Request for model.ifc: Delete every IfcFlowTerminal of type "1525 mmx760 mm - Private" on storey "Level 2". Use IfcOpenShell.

First a look at what the model holds.

```python
import ifcopenshell
import ifcopenshell.util.element

model = ifcopenshell.open("model.ifc")
print(model.schema)
storey = next(s for s in model.by_type("IfcBuildingStorey") if s.Name == "Level 2")
terminals = [e for e in ifcopenshell.util.element.get_decomposition(storey) if e.is_a("IfcFlowTerminal")]
seen = {}
for e in terminals:
    element_type = ifcopenshell.util.element.get_type(e)
    name = element_type.Name if element_type not in (None, e) else None
    seen[name] = seen.get(name, 0) + 1
for name, count in sorted(seen.items(), key=str):
    print(count, "x", name)
```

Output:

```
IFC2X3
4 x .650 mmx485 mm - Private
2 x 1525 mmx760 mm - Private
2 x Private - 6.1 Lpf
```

```python
import ifcopenshell
import ifcopenshell.api.root
import ifcopenshell.util.element

model = ifcopenshell.open("model.ifc")

storey = next(s for s in model.by_type("IfcBuildingStorey") if s.Name == "Level 2")
terminals = [e for e in ifcopenshell.util.element.get_decomposition(storey) if e.is_a("IfcFlowTerminal")]
targets = [e for e in terminals if (t := ifcopenshell.util.element.get_type(e)) not in (None, e) and t.Name == "1525 mmx760 mm - Private"]

for e in targets:
    ifcopenshell.api.root.remove_product(model, product=e)
print(len(targets), "removed")

model.write("model_rev.ifc")
```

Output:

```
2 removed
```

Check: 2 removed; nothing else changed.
